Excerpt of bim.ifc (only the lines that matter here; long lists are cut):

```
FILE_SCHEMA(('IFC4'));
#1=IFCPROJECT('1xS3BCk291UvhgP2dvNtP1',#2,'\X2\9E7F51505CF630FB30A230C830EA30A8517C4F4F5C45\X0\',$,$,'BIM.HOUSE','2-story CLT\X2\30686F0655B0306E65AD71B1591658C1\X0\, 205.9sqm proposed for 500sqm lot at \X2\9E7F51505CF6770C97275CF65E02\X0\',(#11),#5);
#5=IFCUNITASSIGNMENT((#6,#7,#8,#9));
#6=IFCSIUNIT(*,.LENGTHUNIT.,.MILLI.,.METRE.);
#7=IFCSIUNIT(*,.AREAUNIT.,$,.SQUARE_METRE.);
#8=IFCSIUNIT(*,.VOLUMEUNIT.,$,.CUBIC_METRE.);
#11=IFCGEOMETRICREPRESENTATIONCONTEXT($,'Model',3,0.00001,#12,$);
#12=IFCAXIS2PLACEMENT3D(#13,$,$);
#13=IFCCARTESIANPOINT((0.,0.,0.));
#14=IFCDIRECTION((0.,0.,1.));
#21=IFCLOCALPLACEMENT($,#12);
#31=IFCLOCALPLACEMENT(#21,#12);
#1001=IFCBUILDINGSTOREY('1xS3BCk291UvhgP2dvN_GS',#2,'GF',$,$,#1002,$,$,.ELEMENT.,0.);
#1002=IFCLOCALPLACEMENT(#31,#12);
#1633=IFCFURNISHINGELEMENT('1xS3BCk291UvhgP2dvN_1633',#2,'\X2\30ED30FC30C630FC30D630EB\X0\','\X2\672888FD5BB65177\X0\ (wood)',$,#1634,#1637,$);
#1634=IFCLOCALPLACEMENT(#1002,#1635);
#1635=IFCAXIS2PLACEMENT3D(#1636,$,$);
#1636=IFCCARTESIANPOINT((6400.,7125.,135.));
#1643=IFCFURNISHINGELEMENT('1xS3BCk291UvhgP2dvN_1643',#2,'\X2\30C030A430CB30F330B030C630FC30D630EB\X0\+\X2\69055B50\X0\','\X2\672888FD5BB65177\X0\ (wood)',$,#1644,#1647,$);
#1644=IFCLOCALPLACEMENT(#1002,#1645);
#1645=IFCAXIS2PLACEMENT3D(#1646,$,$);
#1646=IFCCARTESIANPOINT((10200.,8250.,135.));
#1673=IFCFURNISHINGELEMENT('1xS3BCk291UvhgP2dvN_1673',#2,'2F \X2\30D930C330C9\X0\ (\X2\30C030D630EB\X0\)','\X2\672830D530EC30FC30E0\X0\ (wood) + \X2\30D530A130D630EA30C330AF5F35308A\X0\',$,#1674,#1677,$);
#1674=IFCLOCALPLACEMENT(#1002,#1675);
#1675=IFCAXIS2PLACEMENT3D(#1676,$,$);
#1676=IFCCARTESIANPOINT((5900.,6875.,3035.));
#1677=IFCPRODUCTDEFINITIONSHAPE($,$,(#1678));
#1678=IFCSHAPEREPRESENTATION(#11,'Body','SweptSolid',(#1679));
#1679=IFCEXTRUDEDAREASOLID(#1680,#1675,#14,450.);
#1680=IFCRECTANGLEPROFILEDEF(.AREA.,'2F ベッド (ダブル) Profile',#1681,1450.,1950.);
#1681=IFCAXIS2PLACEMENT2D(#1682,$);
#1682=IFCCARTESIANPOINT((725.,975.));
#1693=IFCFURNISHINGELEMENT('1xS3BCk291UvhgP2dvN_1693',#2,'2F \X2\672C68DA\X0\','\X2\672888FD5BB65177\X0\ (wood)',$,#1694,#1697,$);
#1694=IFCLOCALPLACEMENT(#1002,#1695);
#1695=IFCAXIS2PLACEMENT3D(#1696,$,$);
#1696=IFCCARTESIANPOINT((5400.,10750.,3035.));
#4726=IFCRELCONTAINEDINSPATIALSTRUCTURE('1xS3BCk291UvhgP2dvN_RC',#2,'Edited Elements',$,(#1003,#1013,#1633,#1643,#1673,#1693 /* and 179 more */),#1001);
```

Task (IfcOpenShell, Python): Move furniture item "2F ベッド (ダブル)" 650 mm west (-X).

```python
import ifcopenshell
import ifcopenshell.api.geometry
import ifcopenshell.util.placement
import ifcopenshell.util.unit

model = ifcopenshell.open("bim.ifc")
unit_scale = ifcopenshell.util.unit.calculate_unit_scale(model)

item = model.by_guid("1xS3BCk291UvhgP2dvN_1673")
matrix = ifcopenshell.util.placement.get_local_placement(item.ObjectPlacement)
matrix[0, 3] -= 0.65 / unit_scale
ifcopenshell.api.geometry.edit_object_placement(model, product=item, matrix=matrix, is_si=False)

print(ifcopenshell.util.placement.get_local_placement(item.ObjectPlacement).round(3) + 0.0)

model.write("bim_rev.ifc")
```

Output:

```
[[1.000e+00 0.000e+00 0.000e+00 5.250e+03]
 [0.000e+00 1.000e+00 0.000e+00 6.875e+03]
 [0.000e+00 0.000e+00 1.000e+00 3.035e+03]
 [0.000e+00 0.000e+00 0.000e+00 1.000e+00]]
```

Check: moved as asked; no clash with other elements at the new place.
